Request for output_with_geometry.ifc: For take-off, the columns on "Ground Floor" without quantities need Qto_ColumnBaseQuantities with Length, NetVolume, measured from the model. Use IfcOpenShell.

First a look at what the model holds.

```python
import ifcopenshell
import ifcopenshell.util.element
import ifcopenshell.util.unit

model = ifcopenshell.open("output_with_geometry.ifc")
print(model.schema)
for unit_type in ("LENGTHUNIT", "AREAUNIT", "VOLUMEUNIT"):
    print(unit_type, ifcopenshell.util.unit.calculate_unit_scale(model, unit_type))
storey = next(s for s in model.by_type("IfcBuildingStorey") if s.Name == "Ground Floor")
columns = [e for e in ifcopenshell.util.element.get_decomposition(storey) if e.is_a("IfcColumn")]
for e in sorted(columns, key=lambda e: e.id()):
    print(e.id(), e.is_a(), e.Name, list(ifcopenshell.util.element.get_psets(e, qtos_only=True)), sep=" | ")
```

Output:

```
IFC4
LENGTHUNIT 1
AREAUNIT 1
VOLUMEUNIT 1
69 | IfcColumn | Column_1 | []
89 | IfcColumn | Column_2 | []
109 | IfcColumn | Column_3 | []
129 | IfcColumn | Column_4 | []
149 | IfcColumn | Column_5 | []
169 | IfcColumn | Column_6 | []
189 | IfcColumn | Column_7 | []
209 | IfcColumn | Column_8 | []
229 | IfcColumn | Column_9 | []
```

```python
import ifcopenshell
import ifcopenshell.api.pset
import ifcopenshell.geom
import ifcopenshell.util.element
import ifcopenshell.util.shape
import ifcopenshell.util.unit

model = ifcopenshell.open("output_with_geometry.ifc")
unit_scale = ifcopenshell.util.unit.calculate_unit_scale(model)
volume_scale = ifcopenshell.util.unit.calculate_unit_scale(model, "VOLUMEUNIT")
settings = ifcopenshell.geom.settings()

storey = next(s for s in model.by_type("IfcBuildingStorey") if s.Name == "Ground Floor")
columns = [e for e in ifcopenshell.util.element.get_decomposition(storey) if e.is_a("IfcColumn")]

for e in sorted(columns, key=lambda e: e.id()):
    if ifcopenshell.util.element.get_psets(e, qtos_only=True, should_inherit=False):
        continue
    # Geometry comes back in metres, in the element's own axes.
    shape = ifcopenshell.geom.create_shape(settings, e)
    values = {
        "Length": ifcopenshell.util.shape.get_z(shape.geometry) / unit_scale,
        "NetVolume": ifcopenshell.util.shape.get_volume(shape.geometry) / volume_scale,
    }
    qto = ifcopenshell.api.pset.add_qto(model, product=e, name="Qto_ColumnBaseQuantities")
    ifcopenshell.api.pset.edit_qto(model, qto=qto, properties=values)
    print(e.id(), {k: round(v, 3) for k, v in values.items()})

model.write("output_with_geometry-out.ifc")
```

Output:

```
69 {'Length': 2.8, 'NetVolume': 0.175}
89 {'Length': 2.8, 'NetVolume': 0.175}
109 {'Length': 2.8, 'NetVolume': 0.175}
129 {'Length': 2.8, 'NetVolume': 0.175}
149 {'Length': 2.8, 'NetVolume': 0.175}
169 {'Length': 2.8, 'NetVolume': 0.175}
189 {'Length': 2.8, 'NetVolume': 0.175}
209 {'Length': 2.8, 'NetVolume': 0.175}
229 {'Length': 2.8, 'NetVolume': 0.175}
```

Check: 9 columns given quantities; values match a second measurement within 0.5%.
